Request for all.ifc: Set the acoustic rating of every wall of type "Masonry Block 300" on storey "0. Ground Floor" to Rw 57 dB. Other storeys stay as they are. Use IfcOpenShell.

First a look at what the model holds.

```python
import ifcopenshell
import ifcopenshell.util.element

model = ifcopenshell.open("all.ifc")
print(model.schema)
storey = next(s for s in model.by_type("IfcBuildingStorey") if s.Name == "0. Ground Floor")
walls = [e for e in ifcopenshell.util.element.get_decomposition(storey) if e.is_a("IfcWall")]
seen = {}
for e in walls:
    element_type = ifcopenshell.util.element.get_type(e)
    key = (element_type.Name if element_type != e and element_type else None, ifcopenshell.util.element.get_pset(e, "Pset_WallCommon", "AcousticRating"))
    seen[key] = seen.get(key, 0) + 1
for (name, value), count in sorted(seen.items(), key=str):
    print(count, "x", name, "|", value)
```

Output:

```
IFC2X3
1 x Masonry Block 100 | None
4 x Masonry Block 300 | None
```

```python
import ifcopenshell
import ifcopenshell.api.pset
import ifcopenshell.util.element

model = ifcopenshell.open("all.ifc")

storey = next(s for s in model.by_type("IfcBuildingStorey") if s.Name == "0. Ground Floor")
walls = [e for e in ifcopenshell.util.element.get_decomposition(storey) if e.is_a("IfcWall")]

count = 0
for e in walls:
    element_type = ifcopenshell.util.element.get_type(e)
    if element_type in (None, e) or element_type.Name != "Masonry Block 300":
        continue
    # add_pset returns the element's existing set when there is one.
    pset = ifcopenshell.api.pset.add_pset(model, product=e, name="Pset_WallCommon")
    ifcopenshell.api.pset.edit_pset(model, pset=pset, properties={"AcousticRating": "Rw 57 dB"})
    count += 1

print(count, "walls updated")

model.write("all_v2.ifc")
```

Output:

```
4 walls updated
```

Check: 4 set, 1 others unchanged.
